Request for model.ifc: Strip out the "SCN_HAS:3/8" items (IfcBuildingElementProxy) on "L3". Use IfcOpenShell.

First a look at what the model holds.

```python
import ifcopenshell
import ifcopenshell.util.element

model = ifcopenshell.open("model.ifc")
print(model.schema)
storey = next(s for s in model.by_type("IfcBuildingStorey") if s.Name == "L3")
proxies = [e for e in ifcopenshell.util.element.get_decomposition(storey) if e.is_a("IfcBuildingElementProxy")]
seen = {}
for e in proxies:
    element_type = ifcopenshell.util.element.get_type(e)
    name = element_type.Name if element_type not in (None, e) else None
    seen[name] = seen.get(name, 0) + 1
for name, count in sorted(seen.items(), key=str):
    print(count, "x", name)
```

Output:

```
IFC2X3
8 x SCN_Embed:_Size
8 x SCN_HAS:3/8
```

```python
import ifcopenshell
import ifcopenshell.api.root
import ifcopenshell.util.element

model = ifcopenshell.open("model.ifc")

storey = next(s for s in model.by_type("IfcBuildingStorey") if s.Name == "L3")
proxies = [e for e in ifcopenshell.util.element.get_decomposition(storey) if e.is_a("IfcBuildingElementProxy")]
targets = [e for e in proxies if (t := ifcopenshell.util.element.get_type(e)) not in (None, e) and t.Name == "SCN_HAS:3/8"]

for e in targets:
    ifcopenshell.api.root.remove_product(model, product=e)
print(len(targets), "removed")

model.write("model_rev.ifc")
```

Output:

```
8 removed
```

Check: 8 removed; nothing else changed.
